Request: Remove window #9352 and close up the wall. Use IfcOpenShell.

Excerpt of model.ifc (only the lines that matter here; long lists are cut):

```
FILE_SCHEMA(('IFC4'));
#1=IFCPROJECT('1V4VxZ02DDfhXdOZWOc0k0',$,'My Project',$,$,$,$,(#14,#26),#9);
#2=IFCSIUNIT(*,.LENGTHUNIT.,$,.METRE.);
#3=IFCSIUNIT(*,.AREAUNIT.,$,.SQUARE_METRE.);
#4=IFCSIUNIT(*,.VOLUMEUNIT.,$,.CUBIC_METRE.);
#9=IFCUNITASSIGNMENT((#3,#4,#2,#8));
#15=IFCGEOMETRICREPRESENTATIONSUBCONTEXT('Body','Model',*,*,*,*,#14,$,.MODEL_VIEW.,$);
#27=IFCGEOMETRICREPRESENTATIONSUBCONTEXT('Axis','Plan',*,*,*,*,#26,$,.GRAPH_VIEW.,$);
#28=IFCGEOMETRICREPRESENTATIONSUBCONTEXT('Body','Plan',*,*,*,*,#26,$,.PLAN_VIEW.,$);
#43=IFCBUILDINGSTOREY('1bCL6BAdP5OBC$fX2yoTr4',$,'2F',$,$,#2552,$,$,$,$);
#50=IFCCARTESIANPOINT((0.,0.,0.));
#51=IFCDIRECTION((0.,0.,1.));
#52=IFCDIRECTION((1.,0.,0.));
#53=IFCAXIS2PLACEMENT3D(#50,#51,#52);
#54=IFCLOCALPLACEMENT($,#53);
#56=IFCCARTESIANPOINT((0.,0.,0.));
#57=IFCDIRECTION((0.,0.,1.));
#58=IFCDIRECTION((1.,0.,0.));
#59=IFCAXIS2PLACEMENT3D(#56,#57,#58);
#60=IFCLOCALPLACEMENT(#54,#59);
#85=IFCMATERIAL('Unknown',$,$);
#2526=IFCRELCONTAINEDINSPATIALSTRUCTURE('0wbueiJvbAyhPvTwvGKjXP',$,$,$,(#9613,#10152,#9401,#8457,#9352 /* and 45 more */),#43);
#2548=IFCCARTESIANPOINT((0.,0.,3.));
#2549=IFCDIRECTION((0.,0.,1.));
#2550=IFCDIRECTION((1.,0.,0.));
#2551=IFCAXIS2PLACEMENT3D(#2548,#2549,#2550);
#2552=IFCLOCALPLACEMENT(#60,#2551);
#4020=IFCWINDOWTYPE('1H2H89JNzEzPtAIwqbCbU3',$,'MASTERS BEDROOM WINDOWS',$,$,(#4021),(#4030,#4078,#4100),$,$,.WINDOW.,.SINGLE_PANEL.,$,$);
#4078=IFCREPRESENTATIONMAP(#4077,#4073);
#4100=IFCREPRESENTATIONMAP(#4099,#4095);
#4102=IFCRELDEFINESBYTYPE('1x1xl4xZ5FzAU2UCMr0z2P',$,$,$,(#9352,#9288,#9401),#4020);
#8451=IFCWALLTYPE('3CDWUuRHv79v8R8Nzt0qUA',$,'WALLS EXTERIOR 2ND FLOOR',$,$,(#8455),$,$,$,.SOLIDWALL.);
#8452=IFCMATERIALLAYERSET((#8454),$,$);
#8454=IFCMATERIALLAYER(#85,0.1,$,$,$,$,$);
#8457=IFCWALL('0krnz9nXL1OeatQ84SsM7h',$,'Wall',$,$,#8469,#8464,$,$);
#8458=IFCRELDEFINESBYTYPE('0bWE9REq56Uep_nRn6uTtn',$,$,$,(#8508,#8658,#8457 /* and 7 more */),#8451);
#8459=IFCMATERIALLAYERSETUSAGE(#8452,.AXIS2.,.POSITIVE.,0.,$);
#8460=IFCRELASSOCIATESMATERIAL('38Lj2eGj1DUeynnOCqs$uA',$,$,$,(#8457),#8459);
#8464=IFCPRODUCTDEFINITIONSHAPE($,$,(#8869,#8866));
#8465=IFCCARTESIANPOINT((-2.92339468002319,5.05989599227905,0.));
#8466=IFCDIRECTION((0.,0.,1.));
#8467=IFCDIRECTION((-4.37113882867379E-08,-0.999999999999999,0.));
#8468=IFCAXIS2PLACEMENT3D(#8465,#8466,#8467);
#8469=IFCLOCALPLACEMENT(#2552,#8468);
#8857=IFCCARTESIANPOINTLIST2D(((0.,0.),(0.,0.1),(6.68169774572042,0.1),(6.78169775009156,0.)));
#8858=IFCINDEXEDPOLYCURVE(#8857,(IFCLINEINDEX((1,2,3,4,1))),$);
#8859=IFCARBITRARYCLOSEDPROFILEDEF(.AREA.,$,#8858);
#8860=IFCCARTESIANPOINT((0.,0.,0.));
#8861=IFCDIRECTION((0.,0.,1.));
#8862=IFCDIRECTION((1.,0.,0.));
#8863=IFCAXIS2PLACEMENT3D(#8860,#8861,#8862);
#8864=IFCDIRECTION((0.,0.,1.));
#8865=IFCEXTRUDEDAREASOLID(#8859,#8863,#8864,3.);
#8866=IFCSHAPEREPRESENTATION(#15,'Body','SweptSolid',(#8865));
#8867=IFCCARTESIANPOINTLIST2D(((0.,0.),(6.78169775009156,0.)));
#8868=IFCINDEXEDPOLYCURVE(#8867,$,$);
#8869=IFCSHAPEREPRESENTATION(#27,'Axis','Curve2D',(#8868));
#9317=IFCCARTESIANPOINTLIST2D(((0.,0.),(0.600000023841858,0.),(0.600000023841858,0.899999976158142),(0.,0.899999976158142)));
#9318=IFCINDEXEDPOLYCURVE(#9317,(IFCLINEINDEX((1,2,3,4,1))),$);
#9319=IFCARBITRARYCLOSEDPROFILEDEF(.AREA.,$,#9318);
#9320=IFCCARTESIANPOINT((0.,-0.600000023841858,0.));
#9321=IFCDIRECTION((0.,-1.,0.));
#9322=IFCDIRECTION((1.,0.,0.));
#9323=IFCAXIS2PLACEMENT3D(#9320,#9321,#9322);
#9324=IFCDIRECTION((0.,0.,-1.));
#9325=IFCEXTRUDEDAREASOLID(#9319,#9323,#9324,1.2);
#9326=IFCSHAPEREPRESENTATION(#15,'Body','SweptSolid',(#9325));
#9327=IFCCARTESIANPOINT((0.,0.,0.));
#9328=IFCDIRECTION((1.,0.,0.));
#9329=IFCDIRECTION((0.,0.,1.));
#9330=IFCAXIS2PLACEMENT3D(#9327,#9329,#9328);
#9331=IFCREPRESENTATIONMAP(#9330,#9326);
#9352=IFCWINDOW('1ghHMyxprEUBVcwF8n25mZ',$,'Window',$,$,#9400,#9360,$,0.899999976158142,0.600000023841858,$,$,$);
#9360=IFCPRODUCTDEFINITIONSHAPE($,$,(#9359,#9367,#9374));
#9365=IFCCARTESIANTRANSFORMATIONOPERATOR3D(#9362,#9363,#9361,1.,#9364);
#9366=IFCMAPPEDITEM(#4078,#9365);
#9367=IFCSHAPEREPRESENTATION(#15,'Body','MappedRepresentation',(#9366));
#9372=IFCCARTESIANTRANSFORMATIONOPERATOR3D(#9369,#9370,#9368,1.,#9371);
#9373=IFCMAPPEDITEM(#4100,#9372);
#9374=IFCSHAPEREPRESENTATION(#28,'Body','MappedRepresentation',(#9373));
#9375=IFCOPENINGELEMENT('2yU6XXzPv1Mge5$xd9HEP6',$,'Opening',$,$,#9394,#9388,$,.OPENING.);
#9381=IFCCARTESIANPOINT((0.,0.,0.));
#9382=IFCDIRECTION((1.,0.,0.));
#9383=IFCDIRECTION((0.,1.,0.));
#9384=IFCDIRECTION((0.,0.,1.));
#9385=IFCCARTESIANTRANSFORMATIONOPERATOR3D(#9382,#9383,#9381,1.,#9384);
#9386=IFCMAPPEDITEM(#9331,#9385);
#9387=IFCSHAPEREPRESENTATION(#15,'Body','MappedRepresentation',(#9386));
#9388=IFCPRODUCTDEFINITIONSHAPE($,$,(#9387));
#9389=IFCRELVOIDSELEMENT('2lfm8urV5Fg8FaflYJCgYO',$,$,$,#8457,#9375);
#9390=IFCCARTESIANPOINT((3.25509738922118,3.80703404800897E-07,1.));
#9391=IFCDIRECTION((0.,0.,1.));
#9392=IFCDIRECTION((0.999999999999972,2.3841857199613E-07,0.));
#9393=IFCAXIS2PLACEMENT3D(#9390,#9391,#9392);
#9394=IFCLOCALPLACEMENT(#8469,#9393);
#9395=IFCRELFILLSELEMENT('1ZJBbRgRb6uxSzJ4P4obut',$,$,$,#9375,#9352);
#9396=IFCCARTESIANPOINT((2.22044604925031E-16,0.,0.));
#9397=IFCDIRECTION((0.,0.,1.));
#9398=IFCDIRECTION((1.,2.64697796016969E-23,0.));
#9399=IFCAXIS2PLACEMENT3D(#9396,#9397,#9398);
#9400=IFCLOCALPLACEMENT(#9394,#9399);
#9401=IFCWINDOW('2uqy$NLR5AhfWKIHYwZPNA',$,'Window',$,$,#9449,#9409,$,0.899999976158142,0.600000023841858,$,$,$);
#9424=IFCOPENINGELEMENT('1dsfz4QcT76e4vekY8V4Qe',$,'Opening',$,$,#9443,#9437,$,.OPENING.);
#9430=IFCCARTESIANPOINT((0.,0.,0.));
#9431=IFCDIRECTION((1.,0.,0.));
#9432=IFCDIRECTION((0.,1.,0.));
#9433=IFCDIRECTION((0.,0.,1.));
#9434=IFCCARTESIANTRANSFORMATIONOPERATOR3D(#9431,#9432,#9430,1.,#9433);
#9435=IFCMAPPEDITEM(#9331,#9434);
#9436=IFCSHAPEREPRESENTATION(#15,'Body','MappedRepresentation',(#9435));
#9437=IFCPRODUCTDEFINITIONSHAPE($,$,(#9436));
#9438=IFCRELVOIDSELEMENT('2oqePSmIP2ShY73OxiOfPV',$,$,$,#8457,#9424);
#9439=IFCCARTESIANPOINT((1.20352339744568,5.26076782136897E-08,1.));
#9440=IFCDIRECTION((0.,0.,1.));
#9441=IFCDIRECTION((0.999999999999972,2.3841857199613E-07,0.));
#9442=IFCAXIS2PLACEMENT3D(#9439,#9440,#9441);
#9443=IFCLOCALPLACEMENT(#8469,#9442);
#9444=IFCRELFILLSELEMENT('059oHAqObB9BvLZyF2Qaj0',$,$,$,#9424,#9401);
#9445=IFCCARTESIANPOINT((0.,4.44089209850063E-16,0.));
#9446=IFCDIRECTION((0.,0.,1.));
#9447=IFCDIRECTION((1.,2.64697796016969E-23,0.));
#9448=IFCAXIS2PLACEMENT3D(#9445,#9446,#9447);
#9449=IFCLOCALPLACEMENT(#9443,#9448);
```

```python
import ifcopenshell
import ifcopenshell.api.feature
import ifcopenshell.api.root
import ifcopenshell.geom
import ifcopenshell.util.shape

model = ifcopenshell.open("model.ifc")
settings = ifcopenshell.geom.settings()


def volume(element):
    """Net volume in cubic metres, openings subtracted."""
    shape = ifcopenshell.geom.create_shape(settings, element)
    return ifcopenshell.util.shape.get_volume(shape.geometry)


window = model.by_guid("1ghHMyxprEUBVcwF8n25mZ")
opening = window.FillsVoids[0].RelatingOpeningElement
wall = opening.VoidsElements[0].RelatingBuildingElement
before = volume(wall)

ifcopenshell.api.root.remove_product(model, product=window)
ifcopenshell.api.feature.remove_feature(model, feature=opening)

after = volume(wall)

print(f"wall volume {before:.3f} -> {after:.3f} m3")

model.write("model-out.ifc")
```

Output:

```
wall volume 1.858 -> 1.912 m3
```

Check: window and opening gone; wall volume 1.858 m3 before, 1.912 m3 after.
